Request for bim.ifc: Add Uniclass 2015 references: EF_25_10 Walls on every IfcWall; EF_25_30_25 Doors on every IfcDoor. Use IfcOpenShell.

First a look at what the model holds.

```python
import ifcopenshell

model = ifcopenshell.open("bim.ifc")
print(model.schema)
print("classifications:", [c.Name for c in model.by_type("IfcClassification")])
for ifc_class in ("IfcDoor", "IfcRoof", "IfcStair", "IfcWall", "IfcWindow"):
    print(ifc_class, len(model.by_type(ifc_class)))
```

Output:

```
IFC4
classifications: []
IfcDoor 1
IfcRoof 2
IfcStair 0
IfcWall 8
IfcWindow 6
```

```python
import ifcopenshell
import ifcopenshell.api.classification

model = ifcopenshell.open("bim.ifc")

system = ifcopenshell.api.classification.add_classification(model, classification="Uniclass 2015")

codes = {
    "IfcWall": ("EF_25_10", "Walls"),
    "IfcDoor": ("EF_25_30_25", "Doors"),
}
for ifc_class, (code, name) in codes.items():
    products = model.by_type(ifc_class)
    ifcopenshell.api.classification.add_reference(
        model, products=products, classification=system, identification=code, name=name
    )
    print(code, len(products))

model.write("bim_updated.ifc")
```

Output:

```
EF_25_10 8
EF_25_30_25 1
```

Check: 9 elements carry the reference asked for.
